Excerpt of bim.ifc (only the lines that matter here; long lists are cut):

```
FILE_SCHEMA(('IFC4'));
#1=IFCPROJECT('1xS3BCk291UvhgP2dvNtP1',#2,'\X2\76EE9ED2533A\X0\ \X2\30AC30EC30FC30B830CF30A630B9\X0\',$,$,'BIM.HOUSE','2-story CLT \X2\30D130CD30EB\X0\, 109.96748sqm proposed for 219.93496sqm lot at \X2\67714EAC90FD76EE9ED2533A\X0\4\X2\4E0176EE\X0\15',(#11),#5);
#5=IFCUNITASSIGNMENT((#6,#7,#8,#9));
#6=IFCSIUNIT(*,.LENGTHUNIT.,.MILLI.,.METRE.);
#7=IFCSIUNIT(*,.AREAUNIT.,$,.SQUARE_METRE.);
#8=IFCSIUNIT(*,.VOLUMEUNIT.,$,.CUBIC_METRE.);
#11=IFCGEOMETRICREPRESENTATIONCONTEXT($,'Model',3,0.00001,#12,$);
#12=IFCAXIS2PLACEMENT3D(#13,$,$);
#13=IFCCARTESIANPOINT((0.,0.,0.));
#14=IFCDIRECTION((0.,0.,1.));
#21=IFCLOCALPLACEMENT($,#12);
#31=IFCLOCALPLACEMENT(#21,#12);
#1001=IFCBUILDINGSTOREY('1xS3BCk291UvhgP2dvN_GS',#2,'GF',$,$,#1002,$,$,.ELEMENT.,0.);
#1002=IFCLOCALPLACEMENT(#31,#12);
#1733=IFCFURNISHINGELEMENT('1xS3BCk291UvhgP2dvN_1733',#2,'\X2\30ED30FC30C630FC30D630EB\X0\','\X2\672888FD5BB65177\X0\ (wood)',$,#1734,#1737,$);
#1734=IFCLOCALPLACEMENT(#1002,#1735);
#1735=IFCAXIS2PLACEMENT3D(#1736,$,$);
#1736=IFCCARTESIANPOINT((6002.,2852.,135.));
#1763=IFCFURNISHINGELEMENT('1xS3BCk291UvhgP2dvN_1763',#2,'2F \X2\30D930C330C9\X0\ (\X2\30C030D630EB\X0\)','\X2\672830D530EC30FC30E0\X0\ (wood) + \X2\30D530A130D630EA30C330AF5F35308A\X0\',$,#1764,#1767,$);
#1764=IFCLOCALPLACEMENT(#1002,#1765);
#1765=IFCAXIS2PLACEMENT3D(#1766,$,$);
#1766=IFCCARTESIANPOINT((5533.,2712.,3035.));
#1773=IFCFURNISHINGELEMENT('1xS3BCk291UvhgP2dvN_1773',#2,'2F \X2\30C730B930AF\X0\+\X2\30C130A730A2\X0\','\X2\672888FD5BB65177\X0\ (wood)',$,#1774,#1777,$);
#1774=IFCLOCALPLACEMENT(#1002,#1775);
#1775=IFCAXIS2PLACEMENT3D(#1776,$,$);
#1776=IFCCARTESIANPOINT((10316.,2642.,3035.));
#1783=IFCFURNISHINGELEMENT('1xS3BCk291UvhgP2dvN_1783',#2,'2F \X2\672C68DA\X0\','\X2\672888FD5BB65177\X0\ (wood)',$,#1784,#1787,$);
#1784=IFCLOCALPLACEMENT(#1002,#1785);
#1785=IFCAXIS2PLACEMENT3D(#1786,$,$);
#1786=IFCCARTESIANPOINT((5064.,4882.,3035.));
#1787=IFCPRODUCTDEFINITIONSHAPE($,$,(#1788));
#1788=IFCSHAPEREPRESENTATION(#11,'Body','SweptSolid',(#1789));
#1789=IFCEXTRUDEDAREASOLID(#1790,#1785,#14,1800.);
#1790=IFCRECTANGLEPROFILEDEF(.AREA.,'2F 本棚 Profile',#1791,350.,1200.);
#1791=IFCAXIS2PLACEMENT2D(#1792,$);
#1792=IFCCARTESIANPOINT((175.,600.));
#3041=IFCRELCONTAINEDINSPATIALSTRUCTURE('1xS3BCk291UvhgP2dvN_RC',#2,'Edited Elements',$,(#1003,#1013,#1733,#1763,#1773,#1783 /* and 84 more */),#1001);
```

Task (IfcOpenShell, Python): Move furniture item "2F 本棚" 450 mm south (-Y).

```python
import ifcopenshell
import ifcopenshell.api.geometry
import ifcopenshell.util.placement

model = ifcopenshell.open("bim.ifc")

item = model.by_guid("1xS3BCk291UvhgP2dvN_1783")
matrix = ifcopenshell.util.placement.get_local_placement(item.ObjectPlacement)
matrix[1, 3] -= 450.0
ifcopenshell.api.geometry.edit_object_placement(model, product=item, matrix=matrix, is_si=False)

print(ifcopenshell.util.placement.get_local_placement(item.ObjectPlacement).round(3) + 0.0)

model.write("bim_v2.ifc")
```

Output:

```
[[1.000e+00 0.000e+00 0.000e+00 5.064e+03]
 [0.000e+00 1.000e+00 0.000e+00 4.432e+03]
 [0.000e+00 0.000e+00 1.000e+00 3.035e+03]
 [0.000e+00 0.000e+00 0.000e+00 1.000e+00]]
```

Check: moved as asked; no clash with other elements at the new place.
